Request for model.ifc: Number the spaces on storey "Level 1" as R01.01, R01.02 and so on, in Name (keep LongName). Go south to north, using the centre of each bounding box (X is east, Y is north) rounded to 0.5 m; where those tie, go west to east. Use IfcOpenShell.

First a look at what the model holds.

```python
import ifcopenshell
import ifcopenshell.util.element
import ifcopenshell.util.placement

model = ifcopenshell.open("model.ifc")
print(model.schema)
storey = next(s for s in model.by_type("IfcBuildingStorey") if s.Name == "Level 1")
spaces = [e for e in ifcopenshell.util.element.get_decomposition(storey) if e.is_a("IfcSpace")]
for e in sorted(spaces, key=lambda e: e.id()):
    origin = ifcopenshell.util.placement.get_local_placement(e.ObjectPlacement)[:3, 3]
    print(e.id(), e.Name, e.LongName, origin.round(2) + 0.0, sep=" | ")
```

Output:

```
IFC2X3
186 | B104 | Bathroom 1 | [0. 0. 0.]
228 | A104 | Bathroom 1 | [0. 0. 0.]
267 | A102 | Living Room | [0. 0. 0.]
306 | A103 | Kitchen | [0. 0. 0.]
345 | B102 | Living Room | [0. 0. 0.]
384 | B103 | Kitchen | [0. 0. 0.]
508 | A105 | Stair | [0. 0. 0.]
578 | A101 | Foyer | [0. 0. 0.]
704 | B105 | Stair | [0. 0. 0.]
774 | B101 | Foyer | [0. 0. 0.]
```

```python
import ifcopenshell
import ifcopenshell.geom
import ifcopenshell.util.element
import ifcopenshell.util.shape

model = ifcopenshell.open("model.ifc")
settings = ifcopenshell.geom.settings()
settings.set("use-world-coords", True)


def centre(element):
    shape = ifcopenshell.geom.create_shape(settings, element)
    return ifcopenshell.util.shape.get_bbox_centroid(shape.geometry)


storey = next(s for s in model.by_type("IfcBuildingStorey") if s.Name == "Level 1")
spaces = [e for e in ifcopenshell.util.element.get_decomposition(storey) if e.is_a("IfcSpace")]

# Insertion points can sit at a corner or the storey origin, so sort by the geometry (in metres).
centres = {e: centre(e) for e in spaces}
spaces.sort(key=lambda e: (round(centres[e][1] / 0.5), centres[e][0]))

for i, e in enumerate(spaces, start=1):
    number = f"R01.{i:02d}"
    e.Name = number
    print(e.id(), number)

model.write("model-out.ifc")
```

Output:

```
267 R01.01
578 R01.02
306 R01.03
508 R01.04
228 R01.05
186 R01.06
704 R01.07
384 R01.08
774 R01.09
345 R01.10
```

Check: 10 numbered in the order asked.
